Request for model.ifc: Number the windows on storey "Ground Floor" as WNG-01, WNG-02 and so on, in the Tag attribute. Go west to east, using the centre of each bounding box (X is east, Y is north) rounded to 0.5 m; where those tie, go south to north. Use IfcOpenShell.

First a look at what the model holds.

```python
import ifcopenshell
import ifcopenshell.util.element
import ifcopenshell.util.placement

model = ifcopenshell.open("model.ifc")
print(model.schema)
storey = next(s for s in model.by_type("IfcBuildingStorey") if s.Name == "Ground Floor")
windows = [e for e in ifcopenshell.util.element.get_decomposition(storey) if e.is_a("IfcWindow")]
for e in sorted(windows, key=lambda e: e.id()):
    origin = ifcopenshell.util.placement.get_local_placement(e.ObjectPlacement)[:3, 3]
    print(e.id(), e.Tag, e.Name, origin.round(2) + 0.0, sep=" | ")
```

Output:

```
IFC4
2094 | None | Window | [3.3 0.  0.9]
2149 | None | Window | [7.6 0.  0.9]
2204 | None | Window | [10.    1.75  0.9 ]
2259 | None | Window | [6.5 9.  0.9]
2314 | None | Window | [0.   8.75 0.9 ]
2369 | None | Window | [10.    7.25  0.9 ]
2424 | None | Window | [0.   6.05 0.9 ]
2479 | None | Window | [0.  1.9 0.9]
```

```python
import ifcopenshell
import ifcopenshell.geom
import ifcopenshell.util.element
import ifcopenshell.util.shape

model = ifcopenshell.open("model.ifc")
settings = ifcopenshell.geom.settings()
settings.set("use-world-coords", True)


def centre(element):
    shape = ifcopenshell.geom.create_shape(settings, element)
    return ifcopenshell.util.shape.get_bbox_centroid(shape.geometry)


storey = next(s for s in model.by_type("IfcBuildingStorey") if s.Name == "Ground Floor")
windows = [e for e in ifcopenshell.util.element.get_decomposition(storey) if e.is_a("IfcWindow")]

# Insertion points can sit at a corner or the storey origin, so sort by the geometry (in metres).
centres = {e: centre(e) for e in windows}
windows.sort(key=lambda e: (round(centres[e][0] / 0.5), centres[e][1]))

for i, e in enumerate(windows, start=1):
    number = f"WNG-{i:02d}"
    e.Tag = number
    print(e.id(), number)

model.write("model_rev.ifc")
```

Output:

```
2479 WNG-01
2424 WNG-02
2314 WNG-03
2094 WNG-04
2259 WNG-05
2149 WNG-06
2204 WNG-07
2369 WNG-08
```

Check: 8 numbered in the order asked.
